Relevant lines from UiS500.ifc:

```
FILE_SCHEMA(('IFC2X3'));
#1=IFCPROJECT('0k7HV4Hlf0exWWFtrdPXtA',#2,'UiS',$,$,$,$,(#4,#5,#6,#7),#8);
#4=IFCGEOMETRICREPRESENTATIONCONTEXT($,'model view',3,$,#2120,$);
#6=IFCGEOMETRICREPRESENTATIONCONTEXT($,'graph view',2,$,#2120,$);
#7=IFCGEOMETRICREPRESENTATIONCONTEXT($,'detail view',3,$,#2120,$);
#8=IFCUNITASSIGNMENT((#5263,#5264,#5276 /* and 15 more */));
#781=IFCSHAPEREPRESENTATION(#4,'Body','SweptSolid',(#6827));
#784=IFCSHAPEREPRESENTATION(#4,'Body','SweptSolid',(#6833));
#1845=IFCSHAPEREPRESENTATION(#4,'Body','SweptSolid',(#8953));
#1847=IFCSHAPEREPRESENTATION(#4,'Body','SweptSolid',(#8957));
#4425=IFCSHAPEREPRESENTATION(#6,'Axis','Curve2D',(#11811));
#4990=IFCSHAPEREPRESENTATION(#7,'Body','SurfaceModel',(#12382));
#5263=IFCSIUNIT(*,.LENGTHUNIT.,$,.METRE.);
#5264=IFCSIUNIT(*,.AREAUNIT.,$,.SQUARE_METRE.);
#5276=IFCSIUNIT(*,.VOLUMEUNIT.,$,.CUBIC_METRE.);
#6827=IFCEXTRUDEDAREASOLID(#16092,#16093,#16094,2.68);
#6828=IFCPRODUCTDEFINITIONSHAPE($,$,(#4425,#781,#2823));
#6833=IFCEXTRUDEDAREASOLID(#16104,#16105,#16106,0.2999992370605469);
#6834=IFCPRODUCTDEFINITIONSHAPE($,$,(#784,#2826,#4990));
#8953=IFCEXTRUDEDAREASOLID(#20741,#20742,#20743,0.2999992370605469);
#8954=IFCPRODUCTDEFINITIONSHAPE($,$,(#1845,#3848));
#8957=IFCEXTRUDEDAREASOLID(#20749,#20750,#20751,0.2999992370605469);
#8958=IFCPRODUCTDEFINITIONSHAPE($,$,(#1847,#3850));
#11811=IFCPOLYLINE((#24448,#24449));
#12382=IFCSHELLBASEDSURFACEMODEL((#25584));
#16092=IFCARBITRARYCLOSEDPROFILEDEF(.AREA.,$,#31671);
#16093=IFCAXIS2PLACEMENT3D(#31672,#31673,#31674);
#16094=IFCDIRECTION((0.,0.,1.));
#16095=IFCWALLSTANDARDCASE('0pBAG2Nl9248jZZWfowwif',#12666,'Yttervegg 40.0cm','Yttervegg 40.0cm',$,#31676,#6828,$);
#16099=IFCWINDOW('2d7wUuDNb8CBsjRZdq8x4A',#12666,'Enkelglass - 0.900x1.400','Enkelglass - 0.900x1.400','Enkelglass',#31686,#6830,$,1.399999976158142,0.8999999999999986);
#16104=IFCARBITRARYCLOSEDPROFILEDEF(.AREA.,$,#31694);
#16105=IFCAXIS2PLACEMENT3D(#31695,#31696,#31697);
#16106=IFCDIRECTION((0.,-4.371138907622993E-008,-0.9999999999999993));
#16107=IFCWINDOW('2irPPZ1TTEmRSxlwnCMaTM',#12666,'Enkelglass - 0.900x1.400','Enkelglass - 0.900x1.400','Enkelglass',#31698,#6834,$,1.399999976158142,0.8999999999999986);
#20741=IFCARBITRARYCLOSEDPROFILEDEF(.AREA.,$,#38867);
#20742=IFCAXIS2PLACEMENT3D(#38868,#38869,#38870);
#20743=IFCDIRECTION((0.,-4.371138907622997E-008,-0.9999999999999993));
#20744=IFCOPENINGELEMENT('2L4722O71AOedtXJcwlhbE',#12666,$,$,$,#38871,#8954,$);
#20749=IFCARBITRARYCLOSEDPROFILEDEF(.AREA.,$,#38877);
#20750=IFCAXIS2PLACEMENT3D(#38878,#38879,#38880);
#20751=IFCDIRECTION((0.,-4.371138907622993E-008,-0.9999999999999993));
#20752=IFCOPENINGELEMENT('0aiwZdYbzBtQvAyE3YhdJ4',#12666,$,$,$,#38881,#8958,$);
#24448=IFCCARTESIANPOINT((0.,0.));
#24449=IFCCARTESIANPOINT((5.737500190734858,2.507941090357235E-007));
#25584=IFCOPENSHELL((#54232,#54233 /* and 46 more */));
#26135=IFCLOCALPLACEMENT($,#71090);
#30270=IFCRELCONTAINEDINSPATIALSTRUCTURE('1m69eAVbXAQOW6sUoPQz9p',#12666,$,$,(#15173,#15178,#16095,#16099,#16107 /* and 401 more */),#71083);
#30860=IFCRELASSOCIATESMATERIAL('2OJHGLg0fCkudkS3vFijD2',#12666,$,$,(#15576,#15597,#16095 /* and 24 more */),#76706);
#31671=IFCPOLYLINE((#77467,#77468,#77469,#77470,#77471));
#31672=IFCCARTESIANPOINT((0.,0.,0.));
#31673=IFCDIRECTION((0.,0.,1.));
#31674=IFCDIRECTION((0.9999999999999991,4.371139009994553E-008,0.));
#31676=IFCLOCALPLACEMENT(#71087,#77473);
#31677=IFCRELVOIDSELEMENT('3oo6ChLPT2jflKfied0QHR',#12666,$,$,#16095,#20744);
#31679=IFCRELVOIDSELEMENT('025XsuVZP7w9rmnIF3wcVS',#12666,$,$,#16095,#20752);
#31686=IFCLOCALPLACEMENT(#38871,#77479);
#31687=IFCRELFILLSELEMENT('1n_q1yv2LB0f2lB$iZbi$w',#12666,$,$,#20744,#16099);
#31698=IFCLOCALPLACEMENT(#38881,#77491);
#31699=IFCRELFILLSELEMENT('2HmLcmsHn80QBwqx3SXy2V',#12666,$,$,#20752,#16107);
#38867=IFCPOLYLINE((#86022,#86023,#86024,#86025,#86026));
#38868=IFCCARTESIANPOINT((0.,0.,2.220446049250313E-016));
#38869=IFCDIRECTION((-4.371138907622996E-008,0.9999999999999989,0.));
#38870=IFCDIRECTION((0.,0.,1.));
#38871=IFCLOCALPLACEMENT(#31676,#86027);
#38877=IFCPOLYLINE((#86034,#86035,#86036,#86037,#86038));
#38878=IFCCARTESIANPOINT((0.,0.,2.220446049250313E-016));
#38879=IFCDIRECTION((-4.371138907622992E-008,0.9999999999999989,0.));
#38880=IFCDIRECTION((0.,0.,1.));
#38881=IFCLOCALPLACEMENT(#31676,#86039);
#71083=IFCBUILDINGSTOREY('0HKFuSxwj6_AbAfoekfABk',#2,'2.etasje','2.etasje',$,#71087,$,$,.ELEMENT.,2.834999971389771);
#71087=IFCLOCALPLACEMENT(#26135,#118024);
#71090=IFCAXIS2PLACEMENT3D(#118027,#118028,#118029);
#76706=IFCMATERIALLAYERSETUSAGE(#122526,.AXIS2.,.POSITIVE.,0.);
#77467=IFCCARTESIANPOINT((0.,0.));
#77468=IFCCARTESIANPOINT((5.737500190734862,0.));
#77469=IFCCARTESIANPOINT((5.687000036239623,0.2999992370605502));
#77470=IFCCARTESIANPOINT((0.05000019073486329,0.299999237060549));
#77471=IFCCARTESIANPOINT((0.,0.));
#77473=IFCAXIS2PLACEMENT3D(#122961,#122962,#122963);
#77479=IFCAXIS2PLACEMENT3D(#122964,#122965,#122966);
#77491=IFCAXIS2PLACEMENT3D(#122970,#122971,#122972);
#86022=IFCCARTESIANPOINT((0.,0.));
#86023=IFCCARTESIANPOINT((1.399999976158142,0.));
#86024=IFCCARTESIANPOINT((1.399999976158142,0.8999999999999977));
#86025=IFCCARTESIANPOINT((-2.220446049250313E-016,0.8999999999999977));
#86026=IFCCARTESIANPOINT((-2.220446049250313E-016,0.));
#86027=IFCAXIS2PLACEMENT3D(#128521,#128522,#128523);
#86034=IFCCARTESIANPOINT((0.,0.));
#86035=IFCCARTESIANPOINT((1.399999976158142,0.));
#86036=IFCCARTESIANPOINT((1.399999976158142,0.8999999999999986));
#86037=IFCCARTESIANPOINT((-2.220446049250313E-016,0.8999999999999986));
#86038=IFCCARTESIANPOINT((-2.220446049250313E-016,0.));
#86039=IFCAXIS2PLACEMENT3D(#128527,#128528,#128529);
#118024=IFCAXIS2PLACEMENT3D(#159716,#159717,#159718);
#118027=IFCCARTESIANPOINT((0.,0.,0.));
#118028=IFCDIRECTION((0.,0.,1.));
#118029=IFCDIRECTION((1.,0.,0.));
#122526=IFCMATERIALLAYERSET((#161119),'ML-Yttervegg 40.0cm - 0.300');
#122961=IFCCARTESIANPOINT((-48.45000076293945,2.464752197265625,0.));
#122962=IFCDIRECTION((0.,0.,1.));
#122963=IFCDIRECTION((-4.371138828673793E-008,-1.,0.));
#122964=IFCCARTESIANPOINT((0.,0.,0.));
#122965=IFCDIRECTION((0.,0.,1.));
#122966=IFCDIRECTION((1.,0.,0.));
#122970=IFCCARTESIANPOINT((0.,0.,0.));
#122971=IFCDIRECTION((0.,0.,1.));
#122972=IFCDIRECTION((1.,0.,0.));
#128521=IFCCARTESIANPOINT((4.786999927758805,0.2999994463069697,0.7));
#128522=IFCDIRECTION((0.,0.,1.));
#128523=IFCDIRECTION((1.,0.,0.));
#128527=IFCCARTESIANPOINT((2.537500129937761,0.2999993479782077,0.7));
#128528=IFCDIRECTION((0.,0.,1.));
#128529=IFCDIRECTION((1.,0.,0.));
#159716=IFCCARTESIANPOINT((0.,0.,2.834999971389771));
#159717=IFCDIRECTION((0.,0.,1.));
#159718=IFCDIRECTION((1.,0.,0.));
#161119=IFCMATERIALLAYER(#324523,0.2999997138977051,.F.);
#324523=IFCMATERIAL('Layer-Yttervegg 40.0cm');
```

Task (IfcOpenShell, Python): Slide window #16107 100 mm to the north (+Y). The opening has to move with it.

```python
import ifcopenshell
import ifcopenshell.api.geometry
import ifcopenshell.util.placement
import ifcopenshell.util.unit

model = ifcopenshell.open("UiS500.ifc")
unit_scale = ifcopenshell.util.unit.calculate_unit_scale(model)

window = model.by_id(16107)
opening = window.FillsVoids[0].RelatingOpeningElement
wall = opening.VoidsElements[0].RelatingBuildingElement

wall_matrix = ifcopenshell.util.placement.get_local_placement(wall.ObjectPlacement)
shift = wall_matrix[:3, 0] * -0.1 / unit_scale
before = ifcopenshell.util.placement.get_local_placement(window.ObjectPlacement)[:3, 3].copy()

# The window is placed relative to its opening, so it follows when the opening moves.
matrix = ifcopenshell.util.placement.get_local_placement(opening.ObjectPlacement)
matrix[:3, 3] += shift
ifcopenshell.api.geometry.edit_object_placement(
    model, product=opening, matrix=matrix, is_si=False, should_transform_children=True
)

after = ifcopenshell.util.placement.get_local_placement(window.ObjectPlacement)[:3, 3]
print("window moved by", (after - before).round(3) + 0.0)

model.write("UiS500_edited.ifc")
```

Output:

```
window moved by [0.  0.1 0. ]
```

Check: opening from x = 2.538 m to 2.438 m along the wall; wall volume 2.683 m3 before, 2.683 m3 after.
